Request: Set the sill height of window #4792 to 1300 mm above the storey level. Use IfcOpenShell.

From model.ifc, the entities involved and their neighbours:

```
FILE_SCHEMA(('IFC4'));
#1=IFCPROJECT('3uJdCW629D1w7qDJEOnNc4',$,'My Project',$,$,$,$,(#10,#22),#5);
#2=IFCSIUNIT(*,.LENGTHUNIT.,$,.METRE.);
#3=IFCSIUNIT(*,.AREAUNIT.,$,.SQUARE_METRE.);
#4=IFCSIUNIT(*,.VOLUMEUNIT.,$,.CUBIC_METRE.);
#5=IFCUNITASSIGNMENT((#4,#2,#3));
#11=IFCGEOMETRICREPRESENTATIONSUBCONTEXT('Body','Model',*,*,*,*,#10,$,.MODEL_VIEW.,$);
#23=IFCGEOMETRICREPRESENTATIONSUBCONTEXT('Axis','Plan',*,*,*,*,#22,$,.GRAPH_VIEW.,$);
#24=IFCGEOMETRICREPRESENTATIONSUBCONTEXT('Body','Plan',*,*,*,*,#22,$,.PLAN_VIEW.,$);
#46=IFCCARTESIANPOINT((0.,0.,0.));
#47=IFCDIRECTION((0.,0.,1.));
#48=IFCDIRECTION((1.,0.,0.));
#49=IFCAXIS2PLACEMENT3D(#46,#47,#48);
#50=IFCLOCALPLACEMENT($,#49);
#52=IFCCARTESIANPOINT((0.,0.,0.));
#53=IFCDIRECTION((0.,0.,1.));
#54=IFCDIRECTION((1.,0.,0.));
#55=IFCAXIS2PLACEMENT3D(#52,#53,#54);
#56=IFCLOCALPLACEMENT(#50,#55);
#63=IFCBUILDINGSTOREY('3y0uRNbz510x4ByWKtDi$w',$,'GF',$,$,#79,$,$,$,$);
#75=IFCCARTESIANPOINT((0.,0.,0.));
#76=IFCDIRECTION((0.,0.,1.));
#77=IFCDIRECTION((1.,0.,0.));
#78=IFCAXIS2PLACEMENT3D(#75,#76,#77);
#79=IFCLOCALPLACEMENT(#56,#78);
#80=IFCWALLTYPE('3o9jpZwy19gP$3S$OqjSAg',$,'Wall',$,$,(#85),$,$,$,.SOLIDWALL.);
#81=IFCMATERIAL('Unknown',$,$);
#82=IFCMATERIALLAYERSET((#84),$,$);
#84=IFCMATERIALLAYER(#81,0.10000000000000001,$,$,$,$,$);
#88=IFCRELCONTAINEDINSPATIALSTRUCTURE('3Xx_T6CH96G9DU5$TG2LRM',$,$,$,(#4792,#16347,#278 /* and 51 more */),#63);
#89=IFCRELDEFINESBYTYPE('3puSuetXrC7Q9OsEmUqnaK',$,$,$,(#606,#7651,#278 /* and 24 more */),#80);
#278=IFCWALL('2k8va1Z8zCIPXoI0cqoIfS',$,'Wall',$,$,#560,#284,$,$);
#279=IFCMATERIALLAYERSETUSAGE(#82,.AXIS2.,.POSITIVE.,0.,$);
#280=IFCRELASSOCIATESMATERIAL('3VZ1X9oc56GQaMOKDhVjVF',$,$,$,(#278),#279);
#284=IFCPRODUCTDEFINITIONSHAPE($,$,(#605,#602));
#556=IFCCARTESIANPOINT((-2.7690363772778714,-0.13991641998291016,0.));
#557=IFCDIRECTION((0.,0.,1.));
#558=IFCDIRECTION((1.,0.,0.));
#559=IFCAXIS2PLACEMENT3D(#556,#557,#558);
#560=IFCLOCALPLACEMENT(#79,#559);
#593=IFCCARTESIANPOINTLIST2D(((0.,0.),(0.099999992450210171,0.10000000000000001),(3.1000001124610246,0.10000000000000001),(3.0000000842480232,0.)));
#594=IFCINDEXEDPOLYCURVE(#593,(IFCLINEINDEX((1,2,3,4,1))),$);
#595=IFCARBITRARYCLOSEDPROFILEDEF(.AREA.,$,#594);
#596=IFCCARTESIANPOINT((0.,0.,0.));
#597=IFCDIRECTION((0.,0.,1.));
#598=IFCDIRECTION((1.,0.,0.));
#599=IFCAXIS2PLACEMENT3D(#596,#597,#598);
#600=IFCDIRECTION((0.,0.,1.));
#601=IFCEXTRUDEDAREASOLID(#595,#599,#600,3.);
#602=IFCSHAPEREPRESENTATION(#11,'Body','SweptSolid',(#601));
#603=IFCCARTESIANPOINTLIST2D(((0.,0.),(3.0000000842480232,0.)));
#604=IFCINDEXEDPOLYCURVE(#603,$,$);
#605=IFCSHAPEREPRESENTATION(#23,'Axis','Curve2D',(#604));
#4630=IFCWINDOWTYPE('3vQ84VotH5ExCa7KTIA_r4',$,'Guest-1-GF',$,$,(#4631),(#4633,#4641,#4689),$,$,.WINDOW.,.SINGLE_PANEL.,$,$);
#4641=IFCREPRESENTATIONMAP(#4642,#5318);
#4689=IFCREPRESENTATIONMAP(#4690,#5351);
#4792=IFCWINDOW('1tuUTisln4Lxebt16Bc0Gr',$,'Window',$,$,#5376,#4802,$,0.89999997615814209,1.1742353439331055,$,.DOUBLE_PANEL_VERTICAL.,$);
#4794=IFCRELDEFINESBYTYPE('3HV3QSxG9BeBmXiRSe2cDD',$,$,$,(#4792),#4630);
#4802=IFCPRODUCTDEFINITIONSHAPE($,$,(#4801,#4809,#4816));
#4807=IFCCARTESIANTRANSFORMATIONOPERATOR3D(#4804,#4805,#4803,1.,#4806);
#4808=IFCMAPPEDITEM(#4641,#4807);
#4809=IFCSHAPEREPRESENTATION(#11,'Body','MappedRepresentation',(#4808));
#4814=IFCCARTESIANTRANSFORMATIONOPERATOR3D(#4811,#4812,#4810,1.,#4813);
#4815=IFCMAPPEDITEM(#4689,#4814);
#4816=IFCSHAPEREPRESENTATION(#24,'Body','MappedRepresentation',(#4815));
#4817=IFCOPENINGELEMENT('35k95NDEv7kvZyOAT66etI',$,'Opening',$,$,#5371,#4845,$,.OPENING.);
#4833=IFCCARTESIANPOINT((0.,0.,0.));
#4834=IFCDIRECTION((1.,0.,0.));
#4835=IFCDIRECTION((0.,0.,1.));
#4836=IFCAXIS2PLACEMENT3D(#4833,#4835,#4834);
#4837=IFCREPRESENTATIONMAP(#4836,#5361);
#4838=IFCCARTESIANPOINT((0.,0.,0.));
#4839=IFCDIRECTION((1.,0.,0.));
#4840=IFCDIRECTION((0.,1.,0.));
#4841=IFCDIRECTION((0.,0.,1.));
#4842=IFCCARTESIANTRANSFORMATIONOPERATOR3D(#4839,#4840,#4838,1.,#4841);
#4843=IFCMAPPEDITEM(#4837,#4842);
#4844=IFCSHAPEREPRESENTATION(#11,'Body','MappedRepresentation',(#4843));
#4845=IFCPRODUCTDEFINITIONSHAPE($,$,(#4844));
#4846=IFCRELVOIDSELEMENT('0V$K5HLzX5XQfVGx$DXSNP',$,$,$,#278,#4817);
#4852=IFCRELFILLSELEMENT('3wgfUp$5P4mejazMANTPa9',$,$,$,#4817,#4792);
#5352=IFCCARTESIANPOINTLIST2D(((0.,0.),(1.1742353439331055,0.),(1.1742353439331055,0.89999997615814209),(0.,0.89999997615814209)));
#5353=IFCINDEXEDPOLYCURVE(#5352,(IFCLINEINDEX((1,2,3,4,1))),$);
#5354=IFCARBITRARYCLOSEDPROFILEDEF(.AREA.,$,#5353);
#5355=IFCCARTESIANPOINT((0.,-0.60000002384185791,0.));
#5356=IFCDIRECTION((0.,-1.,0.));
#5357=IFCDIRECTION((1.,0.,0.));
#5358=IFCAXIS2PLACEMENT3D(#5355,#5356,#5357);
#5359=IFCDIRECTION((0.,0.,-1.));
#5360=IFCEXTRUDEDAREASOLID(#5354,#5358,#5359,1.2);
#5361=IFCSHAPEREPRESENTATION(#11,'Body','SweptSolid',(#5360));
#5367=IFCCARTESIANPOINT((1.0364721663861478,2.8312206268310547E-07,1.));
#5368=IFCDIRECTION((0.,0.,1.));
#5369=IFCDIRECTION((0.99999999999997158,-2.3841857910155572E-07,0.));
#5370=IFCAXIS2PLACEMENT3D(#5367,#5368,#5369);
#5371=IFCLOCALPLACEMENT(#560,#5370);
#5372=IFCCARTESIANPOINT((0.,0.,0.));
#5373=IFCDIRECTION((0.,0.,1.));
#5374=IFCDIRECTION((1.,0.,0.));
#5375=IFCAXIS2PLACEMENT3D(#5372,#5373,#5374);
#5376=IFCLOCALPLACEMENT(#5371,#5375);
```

```python
import numpy as np
import ifcopenshell
import ifcopenshell.api.geometry
import ifcopenshell.geom
import ifcopenshell.util.element
import ifcopenshell.util.placement
import ifcopenshell.util.shape
import ifcopenshell.util.unit

model = ifcopenshell.open("model.ifc")
unit_scale = ifcopenshell.util.unit.calculate_unit_scale(model)

window = model.by_guid("1tuUTisln4Lxebt16Bc0Gr")
opening = window.FillsVoids[0].RelatingOpeningElement
storey = ifcopenshell.util.element.get_container(window, ifc_class="IfcBuildingStorey")
level = ifcopenshell.util.placement.get_local_placement(storey.ObjectPlacement)[2, 3]

# The opening's origin need not be at the sill, so measure its lowest point.
shape = ifcopenshell.geom.create_shape(ifcopenshell.geom.settings(), opening)
bottom = ifcopenshell.util.shape.get_shape_bottom_elevation(shape, shape.geometry) / unit_scale
dz = level + 1.3 / unit_scale - bottom

shift = np.array([0.0, 0.0, dz])
# The window is placed relative to its opening, so it follows when the opening moves.
matrix = ifcopenshell.util.placement.get_local_placement(opening.ObjectPlacement)
matrix[:3, 3] += shift
ifcopenshell.api.geometry.edit_object_placement(
    model, product=opening, matrix=matrix, is_si=False, should_transform_children=True
)

print(f"moved by {dz * unit_scale:+.3f} m")

model.write("model_rev.ifc")
```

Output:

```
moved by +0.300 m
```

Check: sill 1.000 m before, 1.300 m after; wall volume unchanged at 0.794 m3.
